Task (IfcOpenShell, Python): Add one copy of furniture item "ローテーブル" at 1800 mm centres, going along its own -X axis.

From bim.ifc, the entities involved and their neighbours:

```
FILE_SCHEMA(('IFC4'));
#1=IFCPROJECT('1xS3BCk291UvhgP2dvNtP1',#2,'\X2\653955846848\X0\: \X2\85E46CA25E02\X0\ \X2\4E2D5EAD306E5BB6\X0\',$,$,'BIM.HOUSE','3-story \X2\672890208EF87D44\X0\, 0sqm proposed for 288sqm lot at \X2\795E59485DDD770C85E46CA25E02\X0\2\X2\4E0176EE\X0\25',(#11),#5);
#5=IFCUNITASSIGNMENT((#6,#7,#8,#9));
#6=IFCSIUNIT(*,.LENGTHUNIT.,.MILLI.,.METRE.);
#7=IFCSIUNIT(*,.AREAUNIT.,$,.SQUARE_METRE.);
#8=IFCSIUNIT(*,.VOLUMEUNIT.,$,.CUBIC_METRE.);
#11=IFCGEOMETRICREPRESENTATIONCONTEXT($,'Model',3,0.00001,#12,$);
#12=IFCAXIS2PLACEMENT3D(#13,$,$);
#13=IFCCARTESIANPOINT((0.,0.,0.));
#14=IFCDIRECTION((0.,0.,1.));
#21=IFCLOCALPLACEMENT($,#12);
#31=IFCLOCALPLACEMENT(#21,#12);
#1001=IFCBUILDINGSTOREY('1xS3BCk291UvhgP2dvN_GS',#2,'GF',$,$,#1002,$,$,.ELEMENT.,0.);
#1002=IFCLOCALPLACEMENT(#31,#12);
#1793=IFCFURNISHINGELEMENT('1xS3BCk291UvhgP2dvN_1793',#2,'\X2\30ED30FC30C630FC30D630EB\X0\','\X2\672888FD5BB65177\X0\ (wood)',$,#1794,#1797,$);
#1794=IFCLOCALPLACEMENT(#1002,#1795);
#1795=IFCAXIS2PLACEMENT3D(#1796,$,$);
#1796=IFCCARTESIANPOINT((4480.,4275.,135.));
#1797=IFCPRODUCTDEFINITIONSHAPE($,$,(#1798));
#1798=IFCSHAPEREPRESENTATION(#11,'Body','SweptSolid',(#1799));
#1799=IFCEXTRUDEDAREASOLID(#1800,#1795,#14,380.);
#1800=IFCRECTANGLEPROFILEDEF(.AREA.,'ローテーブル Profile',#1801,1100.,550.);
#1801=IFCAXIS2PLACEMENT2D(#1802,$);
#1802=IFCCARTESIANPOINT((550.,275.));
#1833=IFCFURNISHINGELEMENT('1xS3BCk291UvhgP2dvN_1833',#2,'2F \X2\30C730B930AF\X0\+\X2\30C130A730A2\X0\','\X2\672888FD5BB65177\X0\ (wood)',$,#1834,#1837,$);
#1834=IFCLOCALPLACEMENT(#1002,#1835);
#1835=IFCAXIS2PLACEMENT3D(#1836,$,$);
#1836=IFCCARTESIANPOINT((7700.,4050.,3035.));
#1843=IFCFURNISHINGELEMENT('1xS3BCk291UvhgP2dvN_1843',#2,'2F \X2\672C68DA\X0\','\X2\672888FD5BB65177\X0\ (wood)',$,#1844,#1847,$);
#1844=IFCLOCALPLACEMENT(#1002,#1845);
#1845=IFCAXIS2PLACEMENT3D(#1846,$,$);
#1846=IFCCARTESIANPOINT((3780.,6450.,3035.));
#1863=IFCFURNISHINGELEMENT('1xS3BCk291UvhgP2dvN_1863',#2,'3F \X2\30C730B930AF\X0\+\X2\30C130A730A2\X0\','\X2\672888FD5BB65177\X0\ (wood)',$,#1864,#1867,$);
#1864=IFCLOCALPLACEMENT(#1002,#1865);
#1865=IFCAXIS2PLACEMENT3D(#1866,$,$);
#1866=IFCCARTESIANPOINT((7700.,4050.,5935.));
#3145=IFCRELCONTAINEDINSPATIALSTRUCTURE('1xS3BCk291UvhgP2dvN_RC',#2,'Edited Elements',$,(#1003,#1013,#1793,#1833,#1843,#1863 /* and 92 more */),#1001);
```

```python
import ifcopenshell
import ifcopenshell.api.geometry
import ifcopenshell.api.root
import ifcopenshell.util.element
import ifcopenshell.util.placement

model = ifcopenshell.open("bim.ifc")


def reuse_history(source, copy):
    """copy_class also copies each property set's owner history, people and application; keep the originals."""
    for rel in copy.IsDefinedBy:
        if rel.is_a("IfcRelDefinesByProperties") and (history := rel.RelatingPropertyDefinition.OwnerHistory):
            rel.RelatingPropertyDefinition.OwnerHistory = source.OwnerHistory
            ifcopenshell.util.element.remove_deep2(model, history)


source = model.by_guid("1xS3BCk291UvhgP2dvN_1793")
base = ifcopenshell.util.placement.get_local_placement(source.ObjectPlacement)
step = -base[:3, 0] * 1800.0

for i in range(1, 2):
    copy = ifcopenshell.api.root.copy_class(model, product=source)
    copy.Representation = ifcopenshell.util.element.copy_deep(
        model, source.Representation, exclude=["IfcGeometricRepresentationContext", "IfcRepresentationMap"]
    )
    reuse_history(source, copy)
    matrix = base.copy()
    matrix[:3, 3] += i * step
    print("added at", matrix[:3, 3].round(3) + 0.0)
    ifcopenshell.api.geometry.edit_object_placement(model, product=copy, matrix=matrix, is_si=False)

model.write("bim_rev.ifc")
```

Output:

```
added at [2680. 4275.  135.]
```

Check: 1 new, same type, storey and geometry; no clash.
